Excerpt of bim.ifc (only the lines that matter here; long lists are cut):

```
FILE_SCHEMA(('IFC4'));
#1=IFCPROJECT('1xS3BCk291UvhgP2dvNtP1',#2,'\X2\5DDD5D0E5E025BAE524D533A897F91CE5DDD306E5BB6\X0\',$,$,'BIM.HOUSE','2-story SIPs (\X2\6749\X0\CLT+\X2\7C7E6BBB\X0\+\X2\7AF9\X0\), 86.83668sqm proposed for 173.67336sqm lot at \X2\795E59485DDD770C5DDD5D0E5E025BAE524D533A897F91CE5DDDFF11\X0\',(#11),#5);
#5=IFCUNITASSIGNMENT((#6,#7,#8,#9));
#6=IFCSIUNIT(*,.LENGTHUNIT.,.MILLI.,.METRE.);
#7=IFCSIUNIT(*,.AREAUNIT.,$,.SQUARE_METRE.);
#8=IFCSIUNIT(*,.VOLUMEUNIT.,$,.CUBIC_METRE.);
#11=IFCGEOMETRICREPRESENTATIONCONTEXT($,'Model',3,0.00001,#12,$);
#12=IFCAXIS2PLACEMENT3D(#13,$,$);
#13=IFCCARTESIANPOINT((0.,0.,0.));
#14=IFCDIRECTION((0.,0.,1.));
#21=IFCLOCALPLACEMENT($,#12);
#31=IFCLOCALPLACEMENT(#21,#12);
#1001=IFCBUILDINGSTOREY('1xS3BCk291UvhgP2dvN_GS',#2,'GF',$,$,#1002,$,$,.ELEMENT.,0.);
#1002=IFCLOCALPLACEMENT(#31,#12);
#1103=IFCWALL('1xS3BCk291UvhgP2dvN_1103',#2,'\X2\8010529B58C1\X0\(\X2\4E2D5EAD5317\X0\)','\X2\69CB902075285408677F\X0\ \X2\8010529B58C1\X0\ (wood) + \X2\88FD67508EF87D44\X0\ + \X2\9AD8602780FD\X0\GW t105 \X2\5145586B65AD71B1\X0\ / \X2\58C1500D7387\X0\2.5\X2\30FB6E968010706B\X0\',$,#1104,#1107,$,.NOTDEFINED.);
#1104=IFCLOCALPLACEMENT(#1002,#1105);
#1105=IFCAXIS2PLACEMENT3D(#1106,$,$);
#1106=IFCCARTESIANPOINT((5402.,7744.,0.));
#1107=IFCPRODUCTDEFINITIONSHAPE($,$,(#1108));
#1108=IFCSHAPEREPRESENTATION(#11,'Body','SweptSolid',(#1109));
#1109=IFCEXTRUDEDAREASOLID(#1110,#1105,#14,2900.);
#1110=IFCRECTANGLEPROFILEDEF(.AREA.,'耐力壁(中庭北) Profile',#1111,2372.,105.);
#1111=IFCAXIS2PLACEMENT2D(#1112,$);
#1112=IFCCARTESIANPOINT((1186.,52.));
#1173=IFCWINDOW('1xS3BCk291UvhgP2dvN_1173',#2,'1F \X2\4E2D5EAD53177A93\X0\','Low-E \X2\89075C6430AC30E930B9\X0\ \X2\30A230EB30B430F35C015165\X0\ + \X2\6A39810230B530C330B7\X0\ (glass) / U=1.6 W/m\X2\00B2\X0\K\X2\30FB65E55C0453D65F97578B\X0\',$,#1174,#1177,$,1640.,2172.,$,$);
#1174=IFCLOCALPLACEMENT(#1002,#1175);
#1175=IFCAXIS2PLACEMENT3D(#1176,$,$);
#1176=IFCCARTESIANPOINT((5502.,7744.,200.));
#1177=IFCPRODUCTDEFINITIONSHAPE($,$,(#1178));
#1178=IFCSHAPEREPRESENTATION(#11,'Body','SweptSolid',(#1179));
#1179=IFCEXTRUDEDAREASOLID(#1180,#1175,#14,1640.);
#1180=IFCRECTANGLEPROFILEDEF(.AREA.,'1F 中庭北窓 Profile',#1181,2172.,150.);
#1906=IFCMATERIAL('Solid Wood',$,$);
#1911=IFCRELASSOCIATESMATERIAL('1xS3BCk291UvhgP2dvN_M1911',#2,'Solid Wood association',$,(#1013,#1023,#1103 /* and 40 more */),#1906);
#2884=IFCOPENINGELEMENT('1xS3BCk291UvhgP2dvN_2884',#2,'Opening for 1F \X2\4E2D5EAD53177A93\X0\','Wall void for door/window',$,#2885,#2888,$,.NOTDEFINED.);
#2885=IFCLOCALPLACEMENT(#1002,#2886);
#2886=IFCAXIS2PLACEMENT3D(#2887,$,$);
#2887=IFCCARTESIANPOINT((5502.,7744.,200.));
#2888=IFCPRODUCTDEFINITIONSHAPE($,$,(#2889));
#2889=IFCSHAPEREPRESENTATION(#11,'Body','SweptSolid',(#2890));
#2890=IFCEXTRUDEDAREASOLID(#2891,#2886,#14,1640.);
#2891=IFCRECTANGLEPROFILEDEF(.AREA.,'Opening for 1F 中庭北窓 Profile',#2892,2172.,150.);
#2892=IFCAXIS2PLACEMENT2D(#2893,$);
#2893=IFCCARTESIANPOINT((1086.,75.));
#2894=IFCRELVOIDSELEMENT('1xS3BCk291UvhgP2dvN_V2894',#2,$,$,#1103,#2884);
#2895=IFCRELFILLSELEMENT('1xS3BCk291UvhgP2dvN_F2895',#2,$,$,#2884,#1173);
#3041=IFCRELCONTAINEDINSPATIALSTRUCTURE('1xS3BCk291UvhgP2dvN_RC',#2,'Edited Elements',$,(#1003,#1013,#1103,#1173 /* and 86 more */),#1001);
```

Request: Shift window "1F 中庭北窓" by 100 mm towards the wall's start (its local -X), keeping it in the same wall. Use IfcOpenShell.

```python
import ifcopenshell
import ifcopenshell.api.geometry
import ifcopenshell.util.placement
import ifcopenshell.util.unit

model = ifcopenshell.open("bim.ifc")
unit_scale = ifcopenshell.util.unit.calculate_unit_scale(model)

window = model.by_id(1173)
opening = window.FillsVoids[0].RelatingOpeningElement
wall = opening.VoidsElements[0].RelatingBuildingElement

wall_matrix = ifcopenshell.util.placement.get_local_placement(wall.ObjectPlacement)
shift = wall_matrix[:3, 0] * -0.1 / unit_scale
before = ifcopenshell.util.placement.get_local_placement(window.ObjectPlacement)[:3, 3].copy()

# The window is not placed relative to its opening, so move both.
for product in (opening, window):
    matrix = ifcopenshell.util.placement.get_local_placement(product.ObjectPlacement)
    matrix[:3, 3] += shift
    ifcopenshell.api.geometry.edit_object_placement(model, product=product, matrix=matrix, is_si=False)

after = ifcopenshell.util.placement.get_local_placement(window.ObjectPlacement)[:3, 3]
print("window moved by", (after - before).round(3) + 0.0)

model.write("bim-out.ifc")
```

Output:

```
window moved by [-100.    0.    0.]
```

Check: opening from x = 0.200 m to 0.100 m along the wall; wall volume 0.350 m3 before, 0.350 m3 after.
